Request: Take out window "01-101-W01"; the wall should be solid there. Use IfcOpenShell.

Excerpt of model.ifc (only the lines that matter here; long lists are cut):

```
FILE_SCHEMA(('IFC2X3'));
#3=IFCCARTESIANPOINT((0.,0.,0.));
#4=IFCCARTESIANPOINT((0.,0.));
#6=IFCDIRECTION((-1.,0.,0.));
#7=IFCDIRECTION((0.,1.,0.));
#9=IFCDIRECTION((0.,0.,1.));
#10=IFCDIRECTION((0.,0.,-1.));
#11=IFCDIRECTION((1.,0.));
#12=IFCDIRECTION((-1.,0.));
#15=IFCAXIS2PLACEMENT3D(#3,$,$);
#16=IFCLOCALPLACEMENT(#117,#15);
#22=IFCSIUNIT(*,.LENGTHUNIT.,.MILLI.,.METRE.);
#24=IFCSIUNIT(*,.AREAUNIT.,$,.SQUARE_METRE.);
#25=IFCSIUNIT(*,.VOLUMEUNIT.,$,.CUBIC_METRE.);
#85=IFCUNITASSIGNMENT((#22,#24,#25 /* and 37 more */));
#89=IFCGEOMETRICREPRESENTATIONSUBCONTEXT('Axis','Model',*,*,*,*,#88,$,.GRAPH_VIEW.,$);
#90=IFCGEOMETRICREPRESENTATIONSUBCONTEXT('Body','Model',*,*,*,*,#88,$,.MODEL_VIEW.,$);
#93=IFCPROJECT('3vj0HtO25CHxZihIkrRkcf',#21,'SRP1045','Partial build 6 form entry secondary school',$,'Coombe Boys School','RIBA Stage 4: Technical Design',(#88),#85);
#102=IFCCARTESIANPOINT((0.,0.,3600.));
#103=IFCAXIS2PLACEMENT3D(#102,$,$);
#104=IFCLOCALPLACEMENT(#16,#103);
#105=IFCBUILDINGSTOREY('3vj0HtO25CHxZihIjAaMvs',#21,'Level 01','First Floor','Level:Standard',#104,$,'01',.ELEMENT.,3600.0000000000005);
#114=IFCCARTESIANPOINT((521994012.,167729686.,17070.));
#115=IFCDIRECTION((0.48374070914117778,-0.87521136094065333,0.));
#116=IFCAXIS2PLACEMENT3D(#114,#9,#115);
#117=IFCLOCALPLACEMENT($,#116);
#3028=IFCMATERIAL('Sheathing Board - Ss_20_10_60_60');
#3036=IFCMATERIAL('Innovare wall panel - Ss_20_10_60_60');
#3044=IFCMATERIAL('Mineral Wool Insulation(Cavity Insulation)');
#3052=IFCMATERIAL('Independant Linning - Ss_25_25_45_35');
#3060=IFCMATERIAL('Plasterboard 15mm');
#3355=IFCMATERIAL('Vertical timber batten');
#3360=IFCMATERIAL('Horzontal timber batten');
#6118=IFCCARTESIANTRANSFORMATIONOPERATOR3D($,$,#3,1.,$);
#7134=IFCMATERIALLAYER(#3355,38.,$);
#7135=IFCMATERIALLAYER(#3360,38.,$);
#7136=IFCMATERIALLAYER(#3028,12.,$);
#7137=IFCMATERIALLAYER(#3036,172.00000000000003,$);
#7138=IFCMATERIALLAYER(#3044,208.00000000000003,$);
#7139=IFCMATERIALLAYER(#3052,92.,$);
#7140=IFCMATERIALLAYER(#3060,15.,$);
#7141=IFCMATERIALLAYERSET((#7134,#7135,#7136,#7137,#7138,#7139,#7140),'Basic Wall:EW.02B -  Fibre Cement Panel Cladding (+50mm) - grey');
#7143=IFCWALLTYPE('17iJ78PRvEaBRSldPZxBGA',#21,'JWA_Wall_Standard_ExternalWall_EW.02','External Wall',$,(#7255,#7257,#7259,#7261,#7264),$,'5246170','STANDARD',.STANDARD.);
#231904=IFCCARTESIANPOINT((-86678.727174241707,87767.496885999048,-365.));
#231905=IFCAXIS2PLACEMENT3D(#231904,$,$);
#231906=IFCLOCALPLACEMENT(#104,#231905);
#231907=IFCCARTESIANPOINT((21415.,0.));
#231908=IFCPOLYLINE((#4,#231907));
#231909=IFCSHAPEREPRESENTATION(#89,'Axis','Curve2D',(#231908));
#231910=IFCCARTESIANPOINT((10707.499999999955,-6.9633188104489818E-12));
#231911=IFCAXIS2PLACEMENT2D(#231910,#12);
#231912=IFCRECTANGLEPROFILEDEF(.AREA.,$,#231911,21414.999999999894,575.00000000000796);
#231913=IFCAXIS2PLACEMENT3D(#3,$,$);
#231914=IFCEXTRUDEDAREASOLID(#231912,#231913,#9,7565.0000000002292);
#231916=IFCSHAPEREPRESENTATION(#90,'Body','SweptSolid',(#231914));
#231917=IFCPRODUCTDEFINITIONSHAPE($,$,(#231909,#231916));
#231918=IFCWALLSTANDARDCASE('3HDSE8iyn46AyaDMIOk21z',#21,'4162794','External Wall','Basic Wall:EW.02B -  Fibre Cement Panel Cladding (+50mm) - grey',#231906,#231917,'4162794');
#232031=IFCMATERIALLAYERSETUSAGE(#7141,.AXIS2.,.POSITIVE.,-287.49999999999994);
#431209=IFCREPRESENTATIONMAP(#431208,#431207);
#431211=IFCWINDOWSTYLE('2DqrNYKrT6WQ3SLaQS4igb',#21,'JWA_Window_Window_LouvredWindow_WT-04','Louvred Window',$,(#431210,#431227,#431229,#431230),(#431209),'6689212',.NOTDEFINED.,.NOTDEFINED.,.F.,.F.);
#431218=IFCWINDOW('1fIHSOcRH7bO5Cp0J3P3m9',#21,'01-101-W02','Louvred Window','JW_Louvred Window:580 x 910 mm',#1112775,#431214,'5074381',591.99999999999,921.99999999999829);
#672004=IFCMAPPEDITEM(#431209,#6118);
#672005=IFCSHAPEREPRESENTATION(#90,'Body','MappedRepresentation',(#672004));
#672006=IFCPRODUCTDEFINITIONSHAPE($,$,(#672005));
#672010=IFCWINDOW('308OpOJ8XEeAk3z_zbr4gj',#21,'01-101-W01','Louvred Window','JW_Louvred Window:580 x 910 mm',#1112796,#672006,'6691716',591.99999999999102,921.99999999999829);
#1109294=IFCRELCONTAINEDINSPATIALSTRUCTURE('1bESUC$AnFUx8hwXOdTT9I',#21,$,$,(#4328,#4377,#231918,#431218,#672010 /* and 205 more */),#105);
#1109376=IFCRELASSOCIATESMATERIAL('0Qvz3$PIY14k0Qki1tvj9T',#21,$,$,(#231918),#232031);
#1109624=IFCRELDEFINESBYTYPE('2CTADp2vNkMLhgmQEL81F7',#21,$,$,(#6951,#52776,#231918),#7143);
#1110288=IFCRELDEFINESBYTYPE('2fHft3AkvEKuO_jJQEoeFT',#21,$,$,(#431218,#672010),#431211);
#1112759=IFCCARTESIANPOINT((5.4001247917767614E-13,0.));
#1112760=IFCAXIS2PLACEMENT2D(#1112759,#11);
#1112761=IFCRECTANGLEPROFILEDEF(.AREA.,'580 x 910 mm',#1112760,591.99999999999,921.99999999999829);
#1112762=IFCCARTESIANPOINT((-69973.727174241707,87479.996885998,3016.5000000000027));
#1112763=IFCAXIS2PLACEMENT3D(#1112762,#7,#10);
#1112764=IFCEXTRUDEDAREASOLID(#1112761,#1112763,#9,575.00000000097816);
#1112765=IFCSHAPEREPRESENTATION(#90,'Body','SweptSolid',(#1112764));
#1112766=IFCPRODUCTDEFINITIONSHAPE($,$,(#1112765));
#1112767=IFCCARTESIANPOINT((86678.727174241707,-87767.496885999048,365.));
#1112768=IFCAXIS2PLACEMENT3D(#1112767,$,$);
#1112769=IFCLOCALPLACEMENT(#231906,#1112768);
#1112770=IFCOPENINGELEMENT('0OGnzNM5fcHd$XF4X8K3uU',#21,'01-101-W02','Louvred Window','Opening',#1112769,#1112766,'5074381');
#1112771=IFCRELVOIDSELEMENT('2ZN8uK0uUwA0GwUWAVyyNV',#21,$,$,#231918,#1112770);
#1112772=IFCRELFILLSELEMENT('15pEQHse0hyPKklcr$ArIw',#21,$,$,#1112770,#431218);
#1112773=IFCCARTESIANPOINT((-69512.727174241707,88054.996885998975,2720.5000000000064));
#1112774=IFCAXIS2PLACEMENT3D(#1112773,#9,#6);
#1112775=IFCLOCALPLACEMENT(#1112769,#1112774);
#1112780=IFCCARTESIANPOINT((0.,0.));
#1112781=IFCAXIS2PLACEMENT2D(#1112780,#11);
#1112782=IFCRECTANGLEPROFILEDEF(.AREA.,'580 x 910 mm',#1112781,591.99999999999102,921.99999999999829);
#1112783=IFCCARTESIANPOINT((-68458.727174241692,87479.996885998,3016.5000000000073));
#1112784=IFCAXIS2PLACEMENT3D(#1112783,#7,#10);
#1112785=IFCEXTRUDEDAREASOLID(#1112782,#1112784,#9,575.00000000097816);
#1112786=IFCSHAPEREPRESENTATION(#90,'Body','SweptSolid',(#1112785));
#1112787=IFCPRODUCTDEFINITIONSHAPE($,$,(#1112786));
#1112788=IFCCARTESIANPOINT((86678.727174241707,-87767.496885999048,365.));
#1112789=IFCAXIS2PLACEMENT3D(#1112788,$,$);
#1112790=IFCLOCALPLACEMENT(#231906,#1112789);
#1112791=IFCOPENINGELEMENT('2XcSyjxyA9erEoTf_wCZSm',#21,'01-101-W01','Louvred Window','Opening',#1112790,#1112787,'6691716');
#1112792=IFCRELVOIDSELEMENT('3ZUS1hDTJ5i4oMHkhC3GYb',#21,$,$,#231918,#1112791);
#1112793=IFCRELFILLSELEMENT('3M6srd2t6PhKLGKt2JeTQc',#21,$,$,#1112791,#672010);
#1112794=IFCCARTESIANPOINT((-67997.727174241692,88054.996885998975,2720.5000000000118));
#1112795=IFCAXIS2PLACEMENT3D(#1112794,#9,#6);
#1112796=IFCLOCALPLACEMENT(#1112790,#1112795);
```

```python
import ifcopenshell
import ifcopenshell.api.feature
import ifcopenshell.api.root
import ifcopenshell.geom
import ifcopenshell.util.shape

model = ifcopenshell.open("model.ifc")
settings = ifcopenshell.geom.settings()


def volume(element):
    """Net volume in cubic metres, openings subtracted."""
    shape = ifcopenshell.geom.create_shape(settings, element)
    return ifcopenshell.util.shape.get_volume(shape.geometry)


window = model.by_guid("308OpOJ8XEeAk3z_zbr4gj")
opening = window.FillsVoids[0].RelatingOpeningElement
wall = opening.VoidsElements[0].RelatingBuildingElement
before = volume(wall)

ifcopenshell.api.root.remove_product(model, product=window)
ifcopenshell.api.feature.remove_feature(model, feature=opening)

after = volume(wall)

print(f"wall volume {before:.3f} -> {after:.3f} m3")

model.write("model_rev.ifc")
```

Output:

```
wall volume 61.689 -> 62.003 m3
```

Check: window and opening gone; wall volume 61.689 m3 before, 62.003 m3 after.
